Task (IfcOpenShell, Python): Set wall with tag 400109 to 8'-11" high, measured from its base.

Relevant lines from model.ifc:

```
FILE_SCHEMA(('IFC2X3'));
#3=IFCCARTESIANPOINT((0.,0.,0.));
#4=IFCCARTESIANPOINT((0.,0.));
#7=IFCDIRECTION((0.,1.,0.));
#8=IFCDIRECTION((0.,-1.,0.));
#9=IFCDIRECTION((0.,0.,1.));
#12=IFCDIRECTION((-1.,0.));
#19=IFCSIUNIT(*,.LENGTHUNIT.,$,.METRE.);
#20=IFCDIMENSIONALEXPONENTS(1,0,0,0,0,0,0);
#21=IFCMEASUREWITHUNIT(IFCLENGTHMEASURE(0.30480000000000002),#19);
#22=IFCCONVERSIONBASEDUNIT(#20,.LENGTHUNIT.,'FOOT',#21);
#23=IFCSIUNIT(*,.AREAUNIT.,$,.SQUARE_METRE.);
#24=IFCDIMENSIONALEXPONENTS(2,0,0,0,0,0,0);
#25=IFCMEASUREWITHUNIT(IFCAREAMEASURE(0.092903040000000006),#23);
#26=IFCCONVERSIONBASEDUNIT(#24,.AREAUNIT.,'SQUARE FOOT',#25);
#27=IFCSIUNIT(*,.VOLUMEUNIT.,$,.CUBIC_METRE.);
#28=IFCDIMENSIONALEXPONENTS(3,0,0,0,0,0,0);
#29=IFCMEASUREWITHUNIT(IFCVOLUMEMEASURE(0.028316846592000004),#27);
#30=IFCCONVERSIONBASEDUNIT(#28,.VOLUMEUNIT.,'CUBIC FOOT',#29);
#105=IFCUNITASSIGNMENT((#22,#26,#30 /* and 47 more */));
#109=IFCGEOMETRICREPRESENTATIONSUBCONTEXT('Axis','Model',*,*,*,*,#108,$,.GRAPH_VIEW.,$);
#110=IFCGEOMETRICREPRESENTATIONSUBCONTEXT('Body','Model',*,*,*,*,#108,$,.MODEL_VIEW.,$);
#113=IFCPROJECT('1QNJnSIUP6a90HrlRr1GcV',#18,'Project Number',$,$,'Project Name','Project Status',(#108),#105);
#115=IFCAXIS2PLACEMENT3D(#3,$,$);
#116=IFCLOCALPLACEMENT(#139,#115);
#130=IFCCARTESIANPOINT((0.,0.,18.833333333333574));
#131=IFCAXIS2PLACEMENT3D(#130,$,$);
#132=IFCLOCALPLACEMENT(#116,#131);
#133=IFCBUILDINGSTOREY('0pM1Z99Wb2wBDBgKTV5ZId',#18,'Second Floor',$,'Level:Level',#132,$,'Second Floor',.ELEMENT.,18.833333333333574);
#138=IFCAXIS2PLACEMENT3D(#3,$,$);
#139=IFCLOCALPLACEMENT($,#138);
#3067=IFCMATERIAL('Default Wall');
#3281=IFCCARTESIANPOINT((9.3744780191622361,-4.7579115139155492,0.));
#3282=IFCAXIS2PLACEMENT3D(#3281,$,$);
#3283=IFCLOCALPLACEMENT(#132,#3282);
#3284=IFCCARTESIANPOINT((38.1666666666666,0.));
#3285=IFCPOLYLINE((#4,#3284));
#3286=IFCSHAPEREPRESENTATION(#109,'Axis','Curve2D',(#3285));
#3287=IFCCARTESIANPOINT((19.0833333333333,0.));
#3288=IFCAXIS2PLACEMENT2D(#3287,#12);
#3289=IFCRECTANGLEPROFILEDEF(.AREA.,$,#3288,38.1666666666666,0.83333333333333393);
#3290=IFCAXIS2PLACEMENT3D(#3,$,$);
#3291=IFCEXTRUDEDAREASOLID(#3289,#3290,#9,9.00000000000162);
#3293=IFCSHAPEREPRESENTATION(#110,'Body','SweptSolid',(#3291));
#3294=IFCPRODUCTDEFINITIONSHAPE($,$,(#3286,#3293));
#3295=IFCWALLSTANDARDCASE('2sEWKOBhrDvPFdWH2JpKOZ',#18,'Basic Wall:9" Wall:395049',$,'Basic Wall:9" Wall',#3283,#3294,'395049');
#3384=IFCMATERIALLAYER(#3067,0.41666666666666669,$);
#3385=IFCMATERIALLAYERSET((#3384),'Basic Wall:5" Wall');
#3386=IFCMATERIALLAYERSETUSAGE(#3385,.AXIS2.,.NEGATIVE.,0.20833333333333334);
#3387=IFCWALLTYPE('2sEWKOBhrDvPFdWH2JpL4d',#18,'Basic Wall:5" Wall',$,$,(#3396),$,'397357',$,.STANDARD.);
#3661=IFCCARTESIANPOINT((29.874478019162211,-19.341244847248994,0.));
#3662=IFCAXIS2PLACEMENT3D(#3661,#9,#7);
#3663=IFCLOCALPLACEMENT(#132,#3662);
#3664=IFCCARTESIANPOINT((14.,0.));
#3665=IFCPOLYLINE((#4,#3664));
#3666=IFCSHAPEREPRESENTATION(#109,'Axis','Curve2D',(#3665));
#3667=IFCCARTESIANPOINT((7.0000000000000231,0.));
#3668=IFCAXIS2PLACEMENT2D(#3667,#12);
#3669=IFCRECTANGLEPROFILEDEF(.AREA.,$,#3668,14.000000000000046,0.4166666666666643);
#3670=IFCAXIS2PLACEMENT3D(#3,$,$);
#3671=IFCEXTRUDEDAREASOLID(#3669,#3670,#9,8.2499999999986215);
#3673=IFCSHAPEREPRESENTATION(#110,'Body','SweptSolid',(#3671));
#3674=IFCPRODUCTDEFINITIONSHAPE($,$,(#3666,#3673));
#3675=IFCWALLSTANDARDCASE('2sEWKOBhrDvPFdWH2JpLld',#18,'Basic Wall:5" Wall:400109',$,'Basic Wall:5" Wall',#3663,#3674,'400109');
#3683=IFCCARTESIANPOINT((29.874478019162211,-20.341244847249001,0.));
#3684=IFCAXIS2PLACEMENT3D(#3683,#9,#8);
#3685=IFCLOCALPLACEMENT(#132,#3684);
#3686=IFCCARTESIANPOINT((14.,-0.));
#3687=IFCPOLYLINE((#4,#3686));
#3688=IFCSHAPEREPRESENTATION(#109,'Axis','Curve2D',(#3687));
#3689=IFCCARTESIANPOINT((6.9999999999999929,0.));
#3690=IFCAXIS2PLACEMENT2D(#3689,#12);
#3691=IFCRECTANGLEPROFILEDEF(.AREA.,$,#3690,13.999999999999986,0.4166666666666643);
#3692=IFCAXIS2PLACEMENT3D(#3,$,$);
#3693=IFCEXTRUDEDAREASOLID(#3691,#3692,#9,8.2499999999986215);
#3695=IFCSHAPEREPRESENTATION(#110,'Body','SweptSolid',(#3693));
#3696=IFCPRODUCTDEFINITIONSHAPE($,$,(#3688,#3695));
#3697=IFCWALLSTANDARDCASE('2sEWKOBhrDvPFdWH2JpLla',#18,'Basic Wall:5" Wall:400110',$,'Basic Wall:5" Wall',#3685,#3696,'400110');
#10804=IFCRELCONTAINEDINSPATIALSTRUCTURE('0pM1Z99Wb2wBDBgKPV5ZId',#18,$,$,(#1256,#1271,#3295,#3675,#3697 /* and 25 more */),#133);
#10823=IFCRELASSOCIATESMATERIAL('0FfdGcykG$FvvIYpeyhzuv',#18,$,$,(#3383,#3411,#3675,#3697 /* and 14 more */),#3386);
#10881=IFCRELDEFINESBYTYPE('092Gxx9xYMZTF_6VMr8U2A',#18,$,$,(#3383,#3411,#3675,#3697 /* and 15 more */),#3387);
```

```python
import ifcopenshell
import ifcopenshell.geom
import ifcopenshell.util.representation
import ifcopenshell.util.shape
import ifcopenshell.util.unit

model = ifcopenshell.open("model.ifc")
unit_scale = ifcopenshell.util.unit.calculate_unit_scale(model)
settings = ifcopenshell.geom.settings()


def volume(element):
    """Net volume in cubic metres, openings subtracted."""
    shape = ifcopenshell.geom.create_shape(settings, element)
    return ifcopenshell.util.shape.get_volume(shape.geometry)


wall = model.by_guid("2sEWKOBhrDvPFdWH2JpLld")
before = volume(wall)

body = ifcopenshell.util.representation.get_representation(wall, "Model", "Body")
solid = body.Items[0]
old_height = solid.Depth
solid.Depth = 107 * 0.0254 / unit_scale
after = volume(wall)

print(f"height {old_height:g} -> {solid.Depth:g}, volume {before:.3f} -> {after:.3f} m3")

model.write("model_edited.ifc")
```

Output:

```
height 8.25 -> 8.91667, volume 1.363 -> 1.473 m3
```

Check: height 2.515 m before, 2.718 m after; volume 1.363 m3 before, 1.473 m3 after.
